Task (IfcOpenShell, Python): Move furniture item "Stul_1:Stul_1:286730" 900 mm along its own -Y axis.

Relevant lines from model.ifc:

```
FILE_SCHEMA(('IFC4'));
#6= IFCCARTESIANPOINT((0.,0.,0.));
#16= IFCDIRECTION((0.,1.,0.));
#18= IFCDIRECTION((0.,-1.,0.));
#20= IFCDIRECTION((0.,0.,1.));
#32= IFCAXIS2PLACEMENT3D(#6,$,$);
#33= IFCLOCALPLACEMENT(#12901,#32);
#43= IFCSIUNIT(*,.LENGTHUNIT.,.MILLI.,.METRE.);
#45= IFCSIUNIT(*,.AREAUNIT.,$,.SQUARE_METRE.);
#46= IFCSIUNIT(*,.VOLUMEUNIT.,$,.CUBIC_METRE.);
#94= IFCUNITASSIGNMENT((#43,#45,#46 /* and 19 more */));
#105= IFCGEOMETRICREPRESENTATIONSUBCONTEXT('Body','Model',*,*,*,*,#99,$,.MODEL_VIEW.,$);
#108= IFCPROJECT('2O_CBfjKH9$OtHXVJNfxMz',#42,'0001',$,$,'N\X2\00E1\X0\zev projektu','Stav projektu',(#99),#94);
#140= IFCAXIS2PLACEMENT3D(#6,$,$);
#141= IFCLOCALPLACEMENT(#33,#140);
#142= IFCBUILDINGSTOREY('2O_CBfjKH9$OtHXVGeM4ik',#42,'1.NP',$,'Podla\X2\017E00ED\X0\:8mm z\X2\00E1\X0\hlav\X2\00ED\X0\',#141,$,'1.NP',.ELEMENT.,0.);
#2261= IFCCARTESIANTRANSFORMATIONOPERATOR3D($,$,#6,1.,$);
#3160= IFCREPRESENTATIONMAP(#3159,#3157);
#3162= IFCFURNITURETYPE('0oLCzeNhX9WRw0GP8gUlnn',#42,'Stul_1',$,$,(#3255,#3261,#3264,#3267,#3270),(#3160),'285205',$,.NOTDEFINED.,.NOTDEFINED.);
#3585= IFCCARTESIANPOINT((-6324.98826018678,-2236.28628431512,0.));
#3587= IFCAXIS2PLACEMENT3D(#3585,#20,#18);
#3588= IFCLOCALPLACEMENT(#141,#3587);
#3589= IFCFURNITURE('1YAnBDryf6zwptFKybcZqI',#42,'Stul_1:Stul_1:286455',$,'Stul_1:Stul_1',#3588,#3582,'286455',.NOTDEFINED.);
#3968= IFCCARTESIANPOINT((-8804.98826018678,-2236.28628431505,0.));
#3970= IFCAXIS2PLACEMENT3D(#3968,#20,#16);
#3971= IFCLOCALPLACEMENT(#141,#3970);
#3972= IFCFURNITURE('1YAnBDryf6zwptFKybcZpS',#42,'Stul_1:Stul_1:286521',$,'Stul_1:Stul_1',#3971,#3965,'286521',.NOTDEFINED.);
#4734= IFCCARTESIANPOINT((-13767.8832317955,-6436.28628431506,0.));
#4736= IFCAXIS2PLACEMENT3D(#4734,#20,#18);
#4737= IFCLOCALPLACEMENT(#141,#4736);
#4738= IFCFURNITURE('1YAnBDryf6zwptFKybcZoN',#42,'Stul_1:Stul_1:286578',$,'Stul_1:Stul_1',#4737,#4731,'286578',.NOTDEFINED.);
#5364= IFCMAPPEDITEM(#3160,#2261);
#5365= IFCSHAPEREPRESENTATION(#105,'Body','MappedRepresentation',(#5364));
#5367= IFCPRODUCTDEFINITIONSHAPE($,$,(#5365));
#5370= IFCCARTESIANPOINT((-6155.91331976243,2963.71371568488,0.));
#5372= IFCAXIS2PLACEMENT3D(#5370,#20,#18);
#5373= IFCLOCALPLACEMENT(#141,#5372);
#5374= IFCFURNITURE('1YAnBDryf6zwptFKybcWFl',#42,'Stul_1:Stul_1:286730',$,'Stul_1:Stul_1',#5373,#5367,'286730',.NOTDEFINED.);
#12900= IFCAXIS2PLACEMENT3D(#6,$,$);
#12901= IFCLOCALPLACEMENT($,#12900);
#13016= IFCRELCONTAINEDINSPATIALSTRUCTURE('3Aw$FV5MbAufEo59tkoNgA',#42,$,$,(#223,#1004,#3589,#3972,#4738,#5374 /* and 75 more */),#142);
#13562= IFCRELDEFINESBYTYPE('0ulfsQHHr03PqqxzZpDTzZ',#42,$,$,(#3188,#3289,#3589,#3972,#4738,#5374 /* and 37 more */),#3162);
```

```python
import ifcopenshell
import ifcopenshell.api.geometry
import ifcopenshell.util.placement
import ifcopenshell.util.unit

model = ifcopenshell.open("model.ifc")
unit_scale = ifcopenshell.util.unit.calculate_unit_scale(model)

item = model.by_guid("1YAnBDryf6zwptFKybcWFl")
matrix = ifcopenshell.util.placement.get_local_placement(item.ObjectPlacement)
matrix[:3, 3] -= matrix[:3, 1] * 0.9 / unit_scale
ifcopenshell.api.geometry.edit_object_placement(model, product=item, matrix=matrix, is_si=False)

print(ifcopenshell.util.placement.get_local_placement(item.ObjectPlacement).round(3) + 0.0)

model.write("model-out.ifc")
```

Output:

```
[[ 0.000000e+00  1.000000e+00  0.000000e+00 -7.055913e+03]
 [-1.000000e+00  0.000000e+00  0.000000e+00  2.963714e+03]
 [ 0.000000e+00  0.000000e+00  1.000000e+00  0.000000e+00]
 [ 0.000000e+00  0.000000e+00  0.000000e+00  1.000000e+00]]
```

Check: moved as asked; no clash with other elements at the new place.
